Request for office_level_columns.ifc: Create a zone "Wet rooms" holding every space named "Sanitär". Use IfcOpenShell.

First a look at what the model holds.

```python
import ifcopenshell

model = ifcopenshell.open("office_level_columns.ifc")
print(model.schema)
seen = {}
for space in model.by_type("IfcSpace"):
    seen[space.LongName] = seen.get(space.LongName, 0) + 1
for name, count in sorted(seen.items(), key=str):
    print(count, "x", name)
print("zones:", [z.Name for z in model.by_type("IfcZone")][:20])
```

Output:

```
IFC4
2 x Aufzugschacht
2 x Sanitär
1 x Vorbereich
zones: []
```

```python
import ifcopenshell
import ifcopenshell.api.group
import ifcopenshell.api.root

model = ifcopenshell.open("office_level_columns.ifc")

names = {"Sanitär"}
spaces = [s for s in model.by_type("IfcSpace") if s.LongName in names]

zone = ifcopenshell.api.root.create_entity(model, ifc_class="IfcZone", name="Wet rooms")
ifcopenshell.api.group.assign_group(model, products=spaces, group=zone)
print(len(spaces), "spaces in", zone.Name)

model.write("office_level_columns_rev.ifc")
```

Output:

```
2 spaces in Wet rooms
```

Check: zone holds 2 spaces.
